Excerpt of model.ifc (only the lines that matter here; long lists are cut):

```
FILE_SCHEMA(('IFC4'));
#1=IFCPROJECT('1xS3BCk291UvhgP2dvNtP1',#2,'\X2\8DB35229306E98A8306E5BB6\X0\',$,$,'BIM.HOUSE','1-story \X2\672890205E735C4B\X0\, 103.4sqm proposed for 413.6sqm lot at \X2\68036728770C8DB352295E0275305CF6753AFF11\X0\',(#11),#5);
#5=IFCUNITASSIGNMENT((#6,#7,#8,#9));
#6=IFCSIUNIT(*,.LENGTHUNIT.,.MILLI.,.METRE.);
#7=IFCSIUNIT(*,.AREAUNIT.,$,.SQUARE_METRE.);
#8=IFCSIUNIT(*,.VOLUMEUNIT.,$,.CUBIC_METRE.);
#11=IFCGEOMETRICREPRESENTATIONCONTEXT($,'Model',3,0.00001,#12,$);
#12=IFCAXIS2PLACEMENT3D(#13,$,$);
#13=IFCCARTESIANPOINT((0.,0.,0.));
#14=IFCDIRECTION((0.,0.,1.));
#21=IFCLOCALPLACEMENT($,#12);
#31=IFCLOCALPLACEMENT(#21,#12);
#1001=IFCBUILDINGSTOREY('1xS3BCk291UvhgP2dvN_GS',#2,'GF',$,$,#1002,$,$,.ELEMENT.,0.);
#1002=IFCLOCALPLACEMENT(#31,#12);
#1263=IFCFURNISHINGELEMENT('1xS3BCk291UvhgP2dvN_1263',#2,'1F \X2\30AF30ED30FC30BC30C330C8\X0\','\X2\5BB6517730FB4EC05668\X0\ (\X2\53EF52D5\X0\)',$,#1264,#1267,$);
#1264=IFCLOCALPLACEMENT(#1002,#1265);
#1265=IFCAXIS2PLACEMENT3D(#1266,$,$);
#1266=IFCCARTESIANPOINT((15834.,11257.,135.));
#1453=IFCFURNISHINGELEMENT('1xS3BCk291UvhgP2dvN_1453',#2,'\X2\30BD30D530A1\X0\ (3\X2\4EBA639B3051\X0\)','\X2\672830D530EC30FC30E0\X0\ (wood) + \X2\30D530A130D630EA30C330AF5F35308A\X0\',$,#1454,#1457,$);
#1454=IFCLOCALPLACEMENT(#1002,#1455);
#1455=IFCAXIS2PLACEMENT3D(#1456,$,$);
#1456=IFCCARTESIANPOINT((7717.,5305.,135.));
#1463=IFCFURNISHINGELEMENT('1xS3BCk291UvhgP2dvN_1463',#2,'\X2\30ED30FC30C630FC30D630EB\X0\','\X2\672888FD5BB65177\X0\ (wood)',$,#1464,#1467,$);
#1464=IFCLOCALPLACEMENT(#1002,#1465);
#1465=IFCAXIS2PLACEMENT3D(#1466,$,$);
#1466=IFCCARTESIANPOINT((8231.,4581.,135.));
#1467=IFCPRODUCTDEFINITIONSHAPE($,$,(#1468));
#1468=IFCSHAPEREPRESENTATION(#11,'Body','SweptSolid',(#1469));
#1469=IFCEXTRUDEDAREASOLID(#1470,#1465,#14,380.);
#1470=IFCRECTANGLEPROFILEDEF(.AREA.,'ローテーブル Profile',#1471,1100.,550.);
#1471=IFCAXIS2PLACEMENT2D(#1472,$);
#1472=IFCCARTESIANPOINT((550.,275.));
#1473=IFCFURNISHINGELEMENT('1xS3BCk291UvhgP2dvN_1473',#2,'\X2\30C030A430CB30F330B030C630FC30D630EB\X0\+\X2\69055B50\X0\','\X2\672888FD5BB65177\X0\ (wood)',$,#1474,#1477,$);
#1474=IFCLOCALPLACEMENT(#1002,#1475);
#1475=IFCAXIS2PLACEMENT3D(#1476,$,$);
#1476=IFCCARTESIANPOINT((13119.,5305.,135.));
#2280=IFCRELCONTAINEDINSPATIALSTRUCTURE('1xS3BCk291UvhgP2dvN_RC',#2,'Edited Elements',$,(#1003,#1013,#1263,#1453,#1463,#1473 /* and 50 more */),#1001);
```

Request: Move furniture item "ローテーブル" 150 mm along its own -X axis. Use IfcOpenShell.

```python
import ifcopenshell
import ifcopenshell.api.geometry
import ifcopenshell.util.placement

model = ifcopenshell.open("model.ifc")

item = model.by_guid("1xS3BCk291UvhgP2dvN_1463")
matrix = ifcopenshell.util.placement.get_local_placement(item.ObjectPlacement)
matrix[:3, 3] -= matrix[:3, 0] * 150.0
ifcopenshell.api.geometry.edit_object_placement(model, product=item, matrix=matrix, is_si=False)

print(ifcopenshell.util.placement.get_local_placement(item.ObjectPlacement).round(3) + 0.0)

model.write("model_v2.ifc")
```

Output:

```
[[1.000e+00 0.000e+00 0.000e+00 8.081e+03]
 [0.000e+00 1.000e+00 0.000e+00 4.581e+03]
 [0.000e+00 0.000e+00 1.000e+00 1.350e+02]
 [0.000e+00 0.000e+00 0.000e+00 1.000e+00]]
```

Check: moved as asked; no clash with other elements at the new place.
